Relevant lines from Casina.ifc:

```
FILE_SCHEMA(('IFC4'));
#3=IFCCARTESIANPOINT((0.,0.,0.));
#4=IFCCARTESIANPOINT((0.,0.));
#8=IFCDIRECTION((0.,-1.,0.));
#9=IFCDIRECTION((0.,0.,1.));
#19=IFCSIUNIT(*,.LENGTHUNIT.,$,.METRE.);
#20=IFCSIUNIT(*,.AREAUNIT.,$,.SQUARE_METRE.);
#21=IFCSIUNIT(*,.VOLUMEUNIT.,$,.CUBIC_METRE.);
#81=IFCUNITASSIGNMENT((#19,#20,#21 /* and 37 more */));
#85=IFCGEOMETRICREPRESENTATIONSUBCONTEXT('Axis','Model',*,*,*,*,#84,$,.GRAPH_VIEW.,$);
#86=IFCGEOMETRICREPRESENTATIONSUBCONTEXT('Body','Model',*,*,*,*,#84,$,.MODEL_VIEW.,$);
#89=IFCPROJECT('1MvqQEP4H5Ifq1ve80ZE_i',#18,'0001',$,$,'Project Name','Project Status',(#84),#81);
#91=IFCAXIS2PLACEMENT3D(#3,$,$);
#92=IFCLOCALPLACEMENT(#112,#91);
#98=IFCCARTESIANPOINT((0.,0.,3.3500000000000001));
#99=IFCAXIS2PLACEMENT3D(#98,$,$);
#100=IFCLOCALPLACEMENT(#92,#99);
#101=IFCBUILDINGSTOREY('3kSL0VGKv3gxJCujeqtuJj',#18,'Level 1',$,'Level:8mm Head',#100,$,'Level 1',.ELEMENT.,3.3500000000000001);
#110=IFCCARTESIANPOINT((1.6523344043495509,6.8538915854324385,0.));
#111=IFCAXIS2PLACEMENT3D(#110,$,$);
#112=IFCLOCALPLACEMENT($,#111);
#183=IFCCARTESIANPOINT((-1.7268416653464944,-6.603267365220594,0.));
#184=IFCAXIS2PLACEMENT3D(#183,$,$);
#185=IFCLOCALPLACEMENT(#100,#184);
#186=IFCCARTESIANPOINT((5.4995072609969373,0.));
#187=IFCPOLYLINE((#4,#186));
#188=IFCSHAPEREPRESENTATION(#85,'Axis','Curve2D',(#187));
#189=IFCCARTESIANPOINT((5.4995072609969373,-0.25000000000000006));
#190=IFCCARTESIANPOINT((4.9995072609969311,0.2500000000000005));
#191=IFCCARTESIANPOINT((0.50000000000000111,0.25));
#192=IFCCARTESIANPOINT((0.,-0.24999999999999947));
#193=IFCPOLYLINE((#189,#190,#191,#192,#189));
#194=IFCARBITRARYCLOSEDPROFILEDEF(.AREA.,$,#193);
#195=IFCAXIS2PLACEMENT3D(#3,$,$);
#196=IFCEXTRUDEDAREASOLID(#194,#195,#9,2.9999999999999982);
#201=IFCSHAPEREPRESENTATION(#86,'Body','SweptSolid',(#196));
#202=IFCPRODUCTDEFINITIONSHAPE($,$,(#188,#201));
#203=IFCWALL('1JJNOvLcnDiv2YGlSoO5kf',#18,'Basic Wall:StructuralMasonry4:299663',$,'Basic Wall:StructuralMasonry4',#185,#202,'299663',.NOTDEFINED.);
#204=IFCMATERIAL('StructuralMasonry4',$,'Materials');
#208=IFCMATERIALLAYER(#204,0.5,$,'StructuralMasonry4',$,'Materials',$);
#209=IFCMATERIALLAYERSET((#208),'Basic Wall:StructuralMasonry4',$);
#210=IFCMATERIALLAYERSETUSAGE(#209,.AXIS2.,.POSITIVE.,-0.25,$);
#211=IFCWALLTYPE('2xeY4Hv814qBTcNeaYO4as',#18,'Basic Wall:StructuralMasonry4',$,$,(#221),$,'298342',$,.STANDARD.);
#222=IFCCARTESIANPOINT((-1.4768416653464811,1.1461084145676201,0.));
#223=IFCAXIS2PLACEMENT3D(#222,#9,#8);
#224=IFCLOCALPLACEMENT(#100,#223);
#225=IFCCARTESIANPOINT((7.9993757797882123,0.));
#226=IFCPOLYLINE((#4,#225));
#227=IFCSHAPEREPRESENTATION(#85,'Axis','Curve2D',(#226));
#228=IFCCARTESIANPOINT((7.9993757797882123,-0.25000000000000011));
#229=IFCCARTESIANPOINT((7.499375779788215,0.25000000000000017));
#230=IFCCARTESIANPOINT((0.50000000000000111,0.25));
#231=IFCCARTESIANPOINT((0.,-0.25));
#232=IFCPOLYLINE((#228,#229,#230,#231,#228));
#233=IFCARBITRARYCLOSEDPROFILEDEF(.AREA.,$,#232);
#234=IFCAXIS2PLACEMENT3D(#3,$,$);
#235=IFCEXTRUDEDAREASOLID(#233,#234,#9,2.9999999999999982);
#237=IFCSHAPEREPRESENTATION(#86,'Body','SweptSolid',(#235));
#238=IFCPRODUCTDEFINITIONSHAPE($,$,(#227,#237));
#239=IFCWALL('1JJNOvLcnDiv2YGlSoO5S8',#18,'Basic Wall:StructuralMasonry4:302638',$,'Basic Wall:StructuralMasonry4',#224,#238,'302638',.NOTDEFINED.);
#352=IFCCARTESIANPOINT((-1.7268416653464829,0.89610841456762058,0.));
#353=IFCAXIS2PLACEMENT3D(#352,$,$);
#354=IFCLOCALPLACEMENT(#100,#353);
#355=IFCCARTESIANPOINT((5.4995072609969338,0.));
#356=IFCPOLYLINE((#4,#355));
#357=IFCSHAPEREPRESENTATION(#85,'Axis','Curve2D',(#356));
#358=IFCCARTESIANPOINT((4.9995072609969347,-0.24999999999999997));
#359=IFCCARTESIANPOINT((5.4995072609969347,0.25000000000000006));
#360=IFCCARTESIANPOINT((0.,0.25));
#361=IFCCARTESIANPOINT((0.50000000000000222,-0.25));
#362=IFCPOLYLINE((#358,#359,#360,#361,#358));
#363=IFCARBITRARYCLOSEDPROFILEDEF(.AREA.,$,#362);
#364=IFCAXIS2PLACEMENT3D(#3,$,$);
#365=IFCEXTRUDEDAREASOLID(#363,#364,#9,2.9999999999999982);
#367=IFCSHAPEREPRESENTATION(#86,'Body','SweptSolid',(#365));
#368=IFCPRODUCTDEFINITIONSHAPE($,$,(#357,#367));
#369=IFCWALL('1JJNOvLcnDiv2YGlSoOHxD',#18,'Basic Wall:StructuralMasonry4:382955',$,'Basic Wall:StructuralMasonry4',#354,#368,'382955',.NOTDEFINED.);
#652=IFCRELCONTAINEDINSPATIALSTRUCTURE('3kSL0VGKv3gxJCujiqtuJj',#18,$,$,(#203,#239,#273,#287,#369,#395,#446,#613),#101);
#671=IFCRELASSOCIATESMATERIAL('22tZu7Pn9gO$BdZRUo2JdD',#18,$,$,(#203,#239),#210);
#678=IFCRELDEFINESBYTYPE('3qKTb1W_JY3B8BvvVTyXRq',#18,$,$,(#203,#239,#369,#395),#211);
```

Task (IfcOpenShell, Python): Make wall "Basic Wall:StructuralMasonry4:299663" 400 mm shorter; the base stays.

```python
import ifcopenshell
import ifcopenshell.geom
import ifcopenshell.util.representation
import ifcopenshell.util.shape
import ifcopenshell.util.unit

model = ifcopenshell.open("Casina.ifc")
unit_scale = ifcopenshell.util.unit.calculate_unit_scale(model)
settings = ifcopenshell.geom.settings()


def volume(element):
    """Net volume in cubic metres, openings subtracted."""
    shape = ifcopenshell.geom.create_shape(settings, element)
    return ifcopenshell.util.shape.get_volume(shape.geometry)


wall = model.by_id(203)
before = volume(wall)

body = ifcopenshell.util.representation.get_representation(wall, "Model", "Body")
solid = body.Items[0]
old_height = solid.Depth
solid.Depth -= 0.4 / unit_scale
after = volume(wall)

print(f"height {old_height:g} -> {solid.Depth:g}, volume {before:.3f} -> {after:.3f} m3")

model.write("Casina_v2.ifc")
```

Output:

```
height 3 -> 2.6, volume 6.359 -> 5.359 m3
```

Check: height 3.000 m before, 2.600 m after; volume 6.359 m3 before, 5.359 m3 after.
